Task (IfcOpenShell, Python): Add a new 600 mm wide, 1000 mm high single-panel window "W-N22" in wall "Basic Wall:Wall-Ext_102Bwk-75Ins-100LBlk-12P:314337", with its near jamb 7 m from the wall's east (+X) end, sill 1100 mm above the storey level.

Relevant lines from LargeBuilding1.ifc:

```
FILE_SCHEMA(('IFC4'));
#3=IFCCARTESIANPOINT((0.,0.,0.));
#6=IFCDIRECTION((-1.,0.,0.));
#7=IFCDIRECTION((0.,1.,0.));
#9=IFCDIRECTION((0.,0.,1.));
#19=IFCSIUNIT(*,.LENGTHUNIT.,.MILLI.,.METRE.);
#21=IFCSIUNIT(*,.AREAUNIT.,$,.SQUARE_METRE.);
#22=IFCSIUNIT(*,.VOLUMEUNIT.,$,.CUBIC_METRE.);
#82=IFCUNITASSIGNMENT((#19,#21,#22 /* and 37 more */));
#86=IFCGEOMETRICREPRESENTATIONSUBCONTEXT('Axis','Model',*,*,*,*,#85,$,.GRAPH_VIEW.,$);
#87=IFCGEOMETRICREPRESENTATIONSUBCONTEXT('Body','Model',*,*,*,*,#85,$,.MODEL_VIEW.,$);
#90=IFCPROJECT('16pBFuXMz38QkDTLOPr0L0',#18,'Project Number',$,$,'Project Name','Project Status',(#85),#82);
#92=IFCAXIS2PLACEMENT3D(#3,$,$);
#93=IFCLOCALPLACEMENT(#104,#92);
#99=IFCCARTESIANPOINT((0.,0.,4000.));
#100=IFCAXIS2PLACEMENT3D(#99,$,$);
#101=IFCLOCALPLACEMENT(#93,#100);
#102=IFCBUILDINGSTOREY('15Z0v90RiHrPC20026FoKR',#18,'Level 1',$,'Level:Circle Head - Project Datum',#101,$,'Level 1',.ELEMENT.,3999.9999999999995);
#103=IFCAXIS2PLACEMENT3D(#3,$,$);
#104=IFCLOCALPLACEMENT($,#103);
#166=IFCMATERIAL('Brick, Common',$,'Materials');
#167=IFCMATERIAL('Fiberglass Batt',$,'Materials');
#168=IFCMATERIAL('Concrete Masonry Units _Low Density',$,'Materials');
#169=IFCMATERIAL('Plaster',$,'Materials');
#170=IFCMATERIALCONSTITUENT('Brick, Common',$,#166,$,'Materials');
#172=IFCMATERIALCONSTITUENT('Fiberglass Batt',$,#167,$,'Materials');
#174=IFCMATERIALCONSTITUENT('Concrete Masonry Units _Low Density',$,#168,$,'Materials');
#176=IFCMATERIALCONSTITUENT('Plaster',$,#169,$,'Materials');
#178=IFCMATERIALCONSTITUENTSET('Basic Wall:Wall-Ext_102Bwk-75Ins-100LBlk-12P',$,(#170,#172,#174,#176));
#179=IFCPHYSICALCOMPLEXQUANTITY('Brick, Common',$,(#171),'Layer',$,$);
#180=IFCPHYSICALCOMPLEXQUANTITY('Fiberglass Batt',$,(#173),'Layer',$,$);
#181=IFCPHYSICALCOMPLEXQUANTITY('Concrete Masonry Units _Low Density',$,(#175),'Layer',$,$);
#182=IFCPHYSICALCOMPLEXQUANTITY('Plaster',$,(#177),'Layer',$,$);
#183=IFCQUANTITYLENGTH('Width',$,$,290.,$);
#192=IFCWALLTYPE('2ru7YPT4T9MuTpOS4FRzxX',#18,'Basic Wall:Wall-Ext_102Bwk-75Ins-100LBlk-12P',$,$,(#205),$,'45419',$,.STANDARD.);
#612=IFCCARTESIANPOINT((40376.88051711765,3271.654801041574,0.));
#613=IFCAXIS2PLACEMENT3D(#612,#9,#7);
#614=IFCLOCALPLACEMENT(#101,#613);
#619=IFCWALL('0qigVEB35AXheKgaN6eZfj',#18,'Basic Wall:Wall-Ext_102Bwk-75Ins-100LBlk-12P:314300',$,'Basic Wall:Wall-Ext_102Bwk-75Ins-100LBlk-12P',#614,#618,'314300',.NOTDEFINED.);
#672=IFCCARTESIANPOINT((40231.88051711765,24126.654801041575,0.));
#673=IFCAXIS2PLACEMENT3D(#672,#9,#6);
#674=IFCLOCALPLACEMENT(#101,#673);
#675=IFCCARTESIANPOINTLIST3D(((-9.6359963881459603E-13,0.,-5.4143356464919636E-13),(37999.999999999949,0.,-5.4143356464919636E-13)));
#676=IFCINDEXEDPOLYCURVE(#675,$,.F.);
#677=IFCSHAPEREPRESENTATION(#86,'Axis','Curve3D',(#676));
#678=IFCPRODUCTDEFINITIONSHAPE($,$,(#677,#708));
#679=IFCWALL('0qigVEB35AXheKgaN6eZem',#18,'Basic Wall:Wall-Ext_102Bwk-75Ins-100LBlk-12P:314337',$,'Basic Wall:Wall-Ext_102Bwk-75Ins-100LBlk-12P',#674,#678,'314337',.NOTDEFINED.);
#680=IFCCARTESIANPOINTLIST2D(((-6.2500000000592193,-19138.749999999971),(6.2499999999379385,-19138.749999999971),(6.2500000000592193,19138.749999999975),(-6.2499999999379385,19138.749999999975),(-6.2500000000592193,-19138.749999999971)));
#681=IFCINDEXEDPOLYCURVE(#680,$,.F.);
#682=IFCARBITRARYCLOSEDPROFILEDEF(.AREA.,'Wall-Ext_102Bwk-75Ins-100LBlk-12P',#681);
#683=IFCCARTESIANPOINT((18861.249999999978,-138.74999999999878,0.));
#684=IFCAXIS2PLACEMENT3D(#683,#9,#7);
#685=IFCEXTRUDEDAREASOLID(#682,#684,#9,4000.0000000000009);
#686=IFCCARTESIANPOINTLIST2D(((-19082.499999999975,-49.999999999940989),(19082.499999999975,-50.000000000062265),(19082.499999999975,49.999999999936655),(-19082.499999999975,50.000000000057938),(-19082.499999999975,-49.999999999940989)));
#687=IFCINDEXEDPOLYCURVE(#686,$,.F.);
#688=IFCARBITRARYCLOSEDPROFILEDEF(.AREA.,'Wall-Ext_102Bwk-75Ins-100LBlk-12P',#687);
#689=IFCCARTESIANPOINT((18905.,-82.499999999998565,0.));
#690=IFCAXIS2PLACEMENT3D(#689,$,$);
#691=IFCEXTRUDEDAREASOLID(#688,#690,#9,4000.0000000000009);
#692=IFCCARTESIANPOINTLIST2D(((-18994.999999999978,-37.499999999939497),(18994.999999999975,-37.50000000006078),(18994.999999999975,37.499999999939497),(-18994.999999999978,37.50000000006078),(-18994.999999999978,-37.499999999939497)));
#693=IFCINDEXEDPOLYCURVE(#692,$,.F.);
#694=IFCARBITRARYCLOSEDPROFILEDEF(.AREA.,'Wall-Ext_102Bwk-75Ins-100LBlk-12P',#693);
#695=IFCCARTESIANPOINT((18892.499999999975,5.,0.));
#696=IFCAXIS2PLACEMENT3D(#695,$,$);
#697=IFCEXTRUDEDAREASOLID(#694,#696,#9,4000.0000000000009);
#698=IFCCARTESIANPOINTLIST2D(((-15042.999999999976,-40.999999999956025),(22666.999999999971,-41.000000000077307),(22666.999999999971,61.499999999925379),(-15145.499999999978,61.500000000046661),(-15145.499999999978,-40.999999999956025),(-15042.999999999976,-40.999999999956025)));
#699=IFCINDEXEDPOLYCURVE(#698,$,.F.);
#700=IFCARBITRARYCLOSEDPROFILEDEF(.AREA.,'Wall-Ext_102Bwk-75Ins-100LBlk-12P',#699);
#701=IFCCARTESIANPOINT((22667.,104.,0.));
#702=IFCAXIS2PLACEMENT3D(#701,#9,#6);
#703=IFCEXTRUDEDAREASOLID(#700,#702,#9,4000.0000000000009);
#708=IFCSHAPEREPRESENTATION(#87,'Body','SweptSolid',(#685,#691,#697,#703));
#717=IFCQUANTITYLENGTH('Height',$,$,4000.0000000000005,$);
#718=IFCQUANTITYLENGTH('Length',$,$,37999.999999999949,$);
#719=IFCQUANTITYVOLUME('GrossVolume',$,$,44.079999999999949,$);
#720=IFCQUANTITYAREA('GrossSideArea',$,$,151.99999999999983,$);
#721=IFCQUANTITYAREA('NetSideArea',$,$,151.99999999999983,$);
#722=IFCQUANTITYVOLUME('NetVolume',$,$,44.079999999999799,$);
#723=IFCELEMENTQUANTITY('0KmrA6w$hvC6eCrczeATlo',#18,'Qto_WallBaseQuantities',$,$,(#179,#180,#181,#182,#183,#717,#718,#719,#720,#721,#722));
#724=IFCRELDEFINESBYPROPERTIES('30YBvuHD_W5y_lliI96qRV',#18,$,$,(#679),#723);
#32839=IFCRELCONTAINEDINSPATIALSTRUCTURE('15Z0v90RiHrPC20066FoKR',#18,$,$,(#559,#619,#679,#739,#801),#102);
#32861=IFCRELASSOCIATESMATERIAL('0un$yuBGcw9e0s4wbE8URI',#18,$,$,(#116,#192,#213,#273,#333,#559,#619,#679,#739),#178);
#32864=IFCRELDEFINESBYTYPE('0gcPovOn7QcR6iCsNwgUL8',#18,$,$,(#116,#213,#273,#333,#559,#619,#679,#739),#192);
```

```python
import numpy as np
import ifcopenshell
import ifcopenshell.api.feature
import ifcopenshell.api.geometry
import ifcopenshell.api.pset
import ifcopenshell.api.root
import ifcopenshell.api.spatial
import ifcopenshell.geom
import ifcopenshell.util.element
import ifcopenshell.util.placement
import ifcopenshell.util.representation
import ifcopenshell.util.shape
import ifcopenshell.util.unit

model = ifcopenshell.open("LargeBuilding1.ifc")
unit_scale = ifcopenshell.util.unit.calculate_unit_scale(model)
area_scale = ifcopenshell.util.unit.calculate_unit_scale(model, "AREAUNIT")
volume_scale = ifcopenshell.util.unit.calculate_unit_scale(model, "VOLUMEUNIT")
settings = ifcopenshell.geom.settings()


def volume(element):
    """Net volume in cubic metres, openings subtracted."""
    shape = ifcopenshell.geom.create_shape(settings, element)
    return ifcopenshell.util.shape.get_volume(shape.geometry)


wall = model.by_guid("0qigVEB35AXheKgaN6eZem")
storey = ifcopenshell.util.element.get_container(wall, ifc_class="IfcBuildingStorey")
context = ifcopenshell.util.representation.get_context(model, "Model", "Body", "MODEL_VIEW")
before = volume(wall)

width, height, from_end, sill = 0.6, 1, 7, 1.1  # metres

# The wall runs along its own X axis, and the end named is its -X end.
wall_shape = ifcopenshell.geom.create_shape(settings, wall)
x, y, z = ifcopenshell.util.shape.get_vertices(wall_shape.geometry).T
start = x.min() + from_end
face, thickness = float(y.min()), float(y.max() - y.min())
wall_matrix = ifcopenshell.util.placement.get_local_placement(wall.ObjectPlacement)
level = ifcopenshell.util.placement.get_local_placement(storey.ObjectPlacement)[2, 3]


def in_wall(x, y):
    """Placement at x, y metres in the wall's axes, at sill height."""
    matrix = wall_matrix.copy()
    matrix[:, 3] = wall_matrix @ np.array([x / unit_scale, y / unit_scale, 0.0, 1.0])
    matrix[2, 3] = level + sill / unit_scale
    return matrix


# Opening: a box that overshoots both wall faces by 50 mm.
opening = ifcopenshell.api.root.create_entity(model, ifc_class="IfcOpeningElement", predefined_type="OPENING")
box = ifcopenshell.api.geometry.add_wall_representation(
    model, context=context, length=width, height=height, thickness=thickness + 0.1
)
ifcopenshell.api.geometry.assign_representation(model, product=opening, representation=box)
ifcopenshell.api.geometry.edit_object_placement(model, product=opening, matrix=in_wall(start, face - 0.05), is_si=False)
ifcopenshell.api.feature.add_feature(model, feature=opening, element=wall)

window = ifcopenshell.api.root.create_entity(model, ifc_class="IfcWindow", name="W-N22", predefined_type="WINDOW")
window.OverallWidth, window.OverallHeight = width / unit_scale, height / unit_scale
window.PartitioningType = "SINGLE_PANEL"
body = ifcopenshell.api.geometry.add_window_representation(
    model,
    context=context,
    overall_width=window.OverallWidth,
    overall_height=window.OverallHeight,
    partition_type="SINGLE_PANEL",
)
ifcopenshell.api.geometry.assign_representation(model, product=window, representation=body)
ifcopenshell.api.spatial.assign_container(model, products=[window], relating_structure=storey)
ifcopenshell.api.feature.add_filling(model, opening=opening, element=window)

# Centre the window in the wall's thickness.
ifcopenshell.api.geometry.edit_object_placement(model, product=window, matrix=in_wall(start, face), is_si=False)
window_shape = ifcopenshell.geom.create_shape(settings, window)
depth = ifcopenshell.util.shape.get_vertices(window_shape.geometry)[:, 1]
offset = face + thickness / 2 - (depth.min() + depth.max()) / 2
ifcopenshell.api.geometry.edit_object_placement(model, product=window, matrix=in_wall(start, offset), is_si=False)

after = volume(wall)

# Update the wall's stored quantities.
qto = model.by_id(ifcopenshell.util.element.get_pset(wall, "Qto_WallBaseQuantities", should_inherit=False)["id"])
ifcopenshell.api.pset.edit_qto(model, qto=qto, properties={
    "NetSideArea": after / thickness / area_scale,
    "NetVolume": after / volume_scale,
})

print(f"wall volume {before:.3f} -> {after:.3f} m3")

model.write("LargeBuilding1_edited.ifc")
```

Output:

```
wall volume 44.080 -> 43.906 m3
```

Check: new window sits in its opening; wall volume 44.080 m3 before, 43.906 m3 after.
